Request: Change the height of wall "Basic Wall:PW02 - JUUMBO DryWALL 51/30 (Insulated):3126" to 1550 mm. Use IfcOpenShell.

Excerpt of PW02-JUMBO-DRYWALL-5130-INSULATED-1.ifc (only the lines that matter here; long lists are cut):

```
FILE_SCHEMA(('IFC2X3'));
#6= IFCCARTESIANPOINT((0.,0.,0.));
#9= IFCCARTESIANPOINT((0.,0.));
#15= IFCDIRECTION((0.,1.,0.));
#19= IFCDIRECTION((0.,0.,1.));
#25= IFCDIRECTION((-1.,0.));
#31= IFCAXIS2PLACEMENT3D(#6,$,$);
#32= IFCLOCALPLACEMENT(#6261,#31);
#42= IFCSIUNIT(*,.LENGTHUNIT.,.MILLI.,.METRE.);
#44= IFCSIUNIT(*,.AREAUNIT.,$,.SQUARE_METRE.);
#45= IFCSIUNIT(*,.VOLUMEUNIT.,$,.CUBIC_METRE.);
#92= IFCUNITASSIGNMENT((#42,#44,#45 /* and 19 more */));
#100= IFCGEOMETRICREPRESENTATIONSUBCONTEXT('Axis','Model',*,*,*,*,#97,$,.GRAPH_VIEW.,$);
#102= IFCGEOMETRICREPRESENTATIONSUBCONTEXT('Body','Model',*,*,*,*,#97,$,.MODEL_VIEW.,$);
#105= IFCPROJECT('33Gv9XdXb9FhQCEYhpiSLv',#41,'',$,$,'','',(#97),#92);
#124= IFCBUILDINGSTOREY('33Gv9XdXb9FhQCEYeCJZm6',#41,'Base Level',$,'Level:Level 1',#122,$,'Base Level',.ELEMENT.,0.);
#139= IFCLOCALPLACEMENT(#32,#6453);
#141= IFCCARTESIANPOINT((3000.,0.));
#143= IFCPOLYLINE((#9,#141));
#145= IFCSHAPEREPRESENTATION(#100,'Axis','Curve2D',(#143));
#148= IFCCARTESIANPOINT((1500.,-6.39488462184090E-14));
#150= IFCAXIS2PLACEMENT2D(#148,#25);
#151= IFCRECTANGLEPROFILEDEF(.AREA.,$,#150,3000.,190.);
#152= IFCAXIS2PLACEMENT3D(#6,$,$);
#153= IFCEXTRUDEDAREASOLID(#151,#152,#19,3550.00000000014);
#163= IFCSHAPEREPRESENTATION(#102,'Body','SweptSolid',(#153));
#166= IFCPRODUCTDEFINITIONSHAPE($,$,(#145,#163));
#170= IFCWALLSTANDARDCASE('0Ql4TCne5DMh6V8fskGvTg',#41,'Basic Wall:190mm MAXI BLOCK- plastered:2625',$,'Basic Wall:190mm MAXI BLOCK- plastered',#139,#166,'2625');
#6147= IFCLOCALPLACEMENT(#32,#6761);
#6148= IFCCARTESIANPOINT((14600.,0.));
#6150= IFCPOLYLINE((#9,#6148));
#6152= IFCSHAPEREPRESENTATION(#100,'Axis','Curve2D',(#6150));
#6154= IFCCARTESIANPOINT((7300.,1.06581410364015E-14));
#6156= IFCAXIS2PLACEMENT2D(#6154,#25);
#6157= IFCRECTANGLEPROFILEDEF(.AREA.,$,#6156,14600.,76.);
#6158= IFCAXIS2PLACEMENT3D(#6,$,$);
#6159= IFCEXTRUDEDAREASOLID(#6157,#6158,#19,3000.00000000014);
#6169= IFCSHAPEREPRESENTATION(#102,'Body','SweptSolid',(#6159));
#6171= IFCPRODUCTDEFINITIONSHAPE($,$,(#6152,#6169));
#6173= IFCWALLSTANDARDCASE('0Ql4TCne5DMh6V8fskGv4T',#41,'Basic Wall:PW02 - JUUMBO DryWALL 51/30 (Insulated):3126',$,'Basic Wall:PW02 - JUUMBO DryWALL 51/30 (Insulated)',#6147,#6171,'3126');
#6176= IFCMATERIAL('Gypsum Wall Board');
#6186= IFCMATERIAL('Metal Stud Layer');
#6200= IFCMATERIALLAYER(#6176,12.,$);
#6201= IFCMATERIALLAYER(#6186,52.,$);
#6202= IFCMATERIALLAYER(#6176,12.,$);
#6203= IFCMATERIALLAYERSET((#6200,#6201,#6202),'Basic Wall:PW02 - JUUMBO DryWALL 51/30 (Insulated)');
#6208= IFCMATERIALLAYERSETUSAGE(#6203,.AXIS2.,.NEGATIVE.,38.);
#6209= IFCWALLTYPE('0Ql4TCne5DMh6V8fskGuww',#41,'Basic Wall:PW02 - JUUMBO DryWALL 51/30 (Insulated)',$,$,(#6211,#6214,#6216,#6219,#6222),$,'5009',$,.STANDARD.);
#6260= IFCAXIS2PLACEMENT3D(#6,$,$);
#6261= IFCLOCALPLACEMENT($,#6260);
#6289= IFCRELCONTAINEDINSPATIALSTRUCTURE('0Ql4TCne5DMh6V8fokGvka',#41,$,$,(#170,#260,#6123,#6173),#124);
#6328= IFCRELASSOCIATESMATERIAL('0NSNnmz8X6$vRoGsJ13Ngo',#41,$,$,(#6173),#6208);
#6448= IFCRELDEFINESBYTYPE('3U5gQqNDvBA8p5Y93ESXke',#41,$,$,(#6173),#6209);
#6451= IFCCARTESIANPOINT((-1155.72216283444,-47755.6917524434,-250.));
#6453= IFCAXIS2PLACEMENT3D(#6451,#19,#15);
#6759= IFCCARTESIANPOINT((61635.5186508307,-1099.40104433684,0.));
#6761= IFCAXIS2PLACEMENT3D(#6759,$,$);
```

```python
import ifcopenshell
import ifcopenshell.geom
import ifcopenshell.util.representation
import ifcopenshell.util.shape

model = ifcopenshell.open("PW02-JUMBO-DRYWALL-5130-INSULATED-1.ifc")
settings = ifcopenshell.geom.settings()


def volume(element):
    """Net volume in cubic metres, openings subtracted."""
    shape = ifcopenshell.geom.create_shape(settings, element)
    return ifcopenshell.util.shape.get_volume(shape.geometry)


wall = model.by_id(6173)
before = volume(wall)

body = ifcopenshell.util.representation.get_representation(wall, "Model", "Body")
solid = body.Items[0]
old_height = solid.Depth
solid.Depth = 1550.0
after = volume(wall)

print(f"height {old_height:g} -> {solid.Depth:g}, volume {before:.3f} -> {after:.3f} m3")

model.write("PW02-JUMBO-DRYWALL-5130-INSULATED-1_updated.ifc")
```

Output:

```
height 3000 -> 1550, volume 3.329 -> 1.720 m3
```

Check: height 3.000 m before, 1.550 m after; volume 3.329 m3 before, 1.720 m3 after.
